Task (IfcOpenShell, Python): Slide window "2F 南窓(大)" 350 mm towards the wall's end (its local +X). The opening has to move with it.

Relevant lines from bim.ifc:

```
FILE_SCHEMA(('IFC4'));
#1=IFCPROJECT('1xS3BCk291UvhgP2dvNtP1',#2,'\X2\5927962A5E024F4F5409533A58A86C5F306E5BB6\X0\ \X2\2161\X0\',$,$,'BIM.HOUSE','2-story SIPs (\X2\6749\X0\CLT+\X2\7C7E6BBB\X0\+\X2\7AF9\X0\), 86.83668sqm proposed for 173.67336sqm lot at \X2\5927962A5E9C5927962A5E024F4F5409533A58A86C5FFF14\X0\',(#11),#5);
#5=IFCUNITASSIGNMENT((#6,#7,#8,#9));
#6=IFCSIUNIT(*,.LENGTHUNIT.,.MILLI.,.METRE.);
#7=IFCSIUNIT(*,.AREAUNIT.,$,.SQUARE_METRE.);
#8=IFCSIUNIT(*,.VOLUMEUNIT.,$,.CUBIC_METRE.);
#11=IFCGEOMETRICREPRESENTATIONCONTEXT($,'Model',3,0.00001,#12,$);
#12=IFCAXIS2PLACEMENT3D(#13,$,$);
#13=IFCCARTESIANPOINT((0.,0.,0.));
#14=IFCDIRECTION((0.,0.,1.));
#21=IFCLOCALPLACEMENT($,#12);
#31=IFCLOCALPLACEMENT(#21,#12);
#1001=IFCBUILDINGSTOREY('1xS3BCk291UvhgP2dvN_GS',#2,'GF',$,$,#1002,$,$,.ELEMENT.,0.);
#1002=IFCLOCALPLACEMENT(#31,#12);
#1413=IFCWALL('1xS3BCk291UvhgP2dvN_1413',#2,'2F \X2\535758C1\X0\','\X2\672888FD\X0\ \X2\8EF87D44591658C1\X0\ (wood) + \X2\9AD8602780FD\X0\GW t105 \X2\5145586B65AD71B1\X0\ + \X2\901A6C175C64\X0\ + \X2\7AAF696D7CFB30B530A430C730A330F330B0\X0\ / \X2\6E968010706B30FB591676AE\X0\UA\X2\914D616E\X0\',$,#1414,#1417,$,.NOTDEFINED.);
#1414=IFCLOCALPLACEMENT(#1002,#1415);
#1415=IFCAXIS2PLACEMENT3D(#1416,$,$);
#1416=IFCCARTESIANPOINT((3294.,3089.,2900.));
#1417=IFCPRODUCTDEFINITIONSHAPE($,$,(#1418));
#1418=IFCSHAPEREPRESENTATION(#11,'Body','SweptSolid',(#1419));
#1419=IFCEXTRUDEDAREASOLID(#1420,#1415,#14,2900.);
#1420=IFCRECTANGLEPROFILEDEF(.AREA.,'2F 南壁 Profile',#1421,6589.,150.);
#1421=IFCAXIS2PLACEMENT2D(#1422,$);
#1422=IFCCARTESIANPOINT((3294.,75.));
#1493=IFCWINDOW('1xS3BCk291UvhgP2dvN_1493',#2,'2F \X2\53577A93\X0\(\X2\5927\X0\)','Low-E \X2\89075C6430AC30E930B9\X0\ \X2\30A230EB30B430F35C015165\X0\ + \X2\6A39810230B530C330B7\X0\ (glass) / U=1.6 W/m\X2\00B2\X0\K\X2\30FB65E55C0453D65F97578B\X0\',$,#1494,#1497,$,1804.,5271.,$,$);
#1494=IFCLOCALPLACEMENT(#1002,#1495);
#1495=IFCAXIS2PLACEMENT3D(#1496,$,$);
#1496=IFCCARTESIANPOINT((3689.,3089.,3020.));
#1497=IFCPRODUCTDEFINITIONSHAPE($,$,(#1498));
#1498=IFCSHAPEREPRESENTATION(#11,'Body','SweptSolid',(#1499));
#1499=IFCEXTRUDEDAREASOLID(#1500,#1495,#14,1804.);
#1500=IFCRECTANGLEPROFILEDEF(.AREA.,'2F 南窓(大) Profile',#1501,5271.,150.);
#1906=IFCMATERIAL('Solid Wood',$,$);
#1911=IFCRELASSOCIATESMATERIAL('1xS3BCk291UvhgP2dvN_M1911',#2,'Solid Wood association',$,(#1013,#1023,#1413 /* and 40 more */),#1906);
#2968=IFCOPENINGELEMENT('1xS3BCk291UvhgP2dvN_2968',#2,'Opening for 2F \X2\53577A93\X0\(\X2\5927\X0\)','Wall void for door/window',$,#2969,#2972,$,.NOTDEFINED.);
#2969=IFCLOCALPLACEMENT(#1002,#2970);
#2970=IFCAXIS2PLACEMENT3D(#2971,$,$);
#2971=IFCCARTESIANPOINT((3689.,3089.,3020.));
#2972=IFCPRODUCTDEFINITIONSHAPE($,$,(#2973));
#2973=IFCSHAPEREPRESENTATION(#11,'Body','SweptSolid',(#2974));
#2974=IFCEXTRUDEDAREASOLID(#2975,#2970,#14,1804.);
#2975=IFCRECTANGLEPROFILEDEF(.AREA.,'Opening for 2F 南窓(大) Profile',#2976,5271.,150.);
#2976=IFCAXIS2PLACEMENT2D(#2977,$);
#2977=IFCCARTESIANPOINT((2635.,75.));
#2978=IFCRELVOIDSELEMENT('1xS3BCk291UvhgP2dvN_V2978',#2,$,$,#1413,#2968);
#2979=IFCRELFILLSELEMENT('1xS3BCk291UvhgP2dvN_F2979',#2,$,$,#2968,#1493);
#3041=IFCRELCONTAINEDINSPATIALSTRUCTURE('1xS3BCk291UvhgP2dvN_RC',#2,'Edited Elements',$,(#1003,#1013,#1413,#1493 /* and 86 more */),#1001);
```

```python
import ifcopenshell
import ifcopenshell.api.geometry
import ifcopenshell.util.placement

model = ifcopenshell.open("bim.ifc")

window = model.by_guid("1xS3BCk291UvhgP2dvN_1493")
opening = window.FillsVoids[0].RelatingOpeningElement
wall = opening.VoidsElements[0].RelatingBuildingElement

wall_matrix = ifcopenshell.util.placement.get_local_placement(wall.ObjectPlacement)
shift = wall_matrix[:3, 0] * 350.0
before = ifcopenshell.util.placement.get_local_placement(window.ObjectPlacement)[:3, 3].copy()

# The window is not placed relative to its opening, so move both.
for product in (opening, window):
    matrix = ifcopenshell.util.placement.get_local_placement(product.ObjectPlacement)
    matrix[:3, 3] += shift
    ifcopenshell.api.geometry.edit_object_placement(model, product=product, matrix=matrix, is_si=False)

after = ifcopenshell.util.placement.get_local_placement(window.ObjectPlacement)[:3, 3]
print("window moved by", (after - before).round(3) + 0.0)

model.write("bim_v2.ifc")
```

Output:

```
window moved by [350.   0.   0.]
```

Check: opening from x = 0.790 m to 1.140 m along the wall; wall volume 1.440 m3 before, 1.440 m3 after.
